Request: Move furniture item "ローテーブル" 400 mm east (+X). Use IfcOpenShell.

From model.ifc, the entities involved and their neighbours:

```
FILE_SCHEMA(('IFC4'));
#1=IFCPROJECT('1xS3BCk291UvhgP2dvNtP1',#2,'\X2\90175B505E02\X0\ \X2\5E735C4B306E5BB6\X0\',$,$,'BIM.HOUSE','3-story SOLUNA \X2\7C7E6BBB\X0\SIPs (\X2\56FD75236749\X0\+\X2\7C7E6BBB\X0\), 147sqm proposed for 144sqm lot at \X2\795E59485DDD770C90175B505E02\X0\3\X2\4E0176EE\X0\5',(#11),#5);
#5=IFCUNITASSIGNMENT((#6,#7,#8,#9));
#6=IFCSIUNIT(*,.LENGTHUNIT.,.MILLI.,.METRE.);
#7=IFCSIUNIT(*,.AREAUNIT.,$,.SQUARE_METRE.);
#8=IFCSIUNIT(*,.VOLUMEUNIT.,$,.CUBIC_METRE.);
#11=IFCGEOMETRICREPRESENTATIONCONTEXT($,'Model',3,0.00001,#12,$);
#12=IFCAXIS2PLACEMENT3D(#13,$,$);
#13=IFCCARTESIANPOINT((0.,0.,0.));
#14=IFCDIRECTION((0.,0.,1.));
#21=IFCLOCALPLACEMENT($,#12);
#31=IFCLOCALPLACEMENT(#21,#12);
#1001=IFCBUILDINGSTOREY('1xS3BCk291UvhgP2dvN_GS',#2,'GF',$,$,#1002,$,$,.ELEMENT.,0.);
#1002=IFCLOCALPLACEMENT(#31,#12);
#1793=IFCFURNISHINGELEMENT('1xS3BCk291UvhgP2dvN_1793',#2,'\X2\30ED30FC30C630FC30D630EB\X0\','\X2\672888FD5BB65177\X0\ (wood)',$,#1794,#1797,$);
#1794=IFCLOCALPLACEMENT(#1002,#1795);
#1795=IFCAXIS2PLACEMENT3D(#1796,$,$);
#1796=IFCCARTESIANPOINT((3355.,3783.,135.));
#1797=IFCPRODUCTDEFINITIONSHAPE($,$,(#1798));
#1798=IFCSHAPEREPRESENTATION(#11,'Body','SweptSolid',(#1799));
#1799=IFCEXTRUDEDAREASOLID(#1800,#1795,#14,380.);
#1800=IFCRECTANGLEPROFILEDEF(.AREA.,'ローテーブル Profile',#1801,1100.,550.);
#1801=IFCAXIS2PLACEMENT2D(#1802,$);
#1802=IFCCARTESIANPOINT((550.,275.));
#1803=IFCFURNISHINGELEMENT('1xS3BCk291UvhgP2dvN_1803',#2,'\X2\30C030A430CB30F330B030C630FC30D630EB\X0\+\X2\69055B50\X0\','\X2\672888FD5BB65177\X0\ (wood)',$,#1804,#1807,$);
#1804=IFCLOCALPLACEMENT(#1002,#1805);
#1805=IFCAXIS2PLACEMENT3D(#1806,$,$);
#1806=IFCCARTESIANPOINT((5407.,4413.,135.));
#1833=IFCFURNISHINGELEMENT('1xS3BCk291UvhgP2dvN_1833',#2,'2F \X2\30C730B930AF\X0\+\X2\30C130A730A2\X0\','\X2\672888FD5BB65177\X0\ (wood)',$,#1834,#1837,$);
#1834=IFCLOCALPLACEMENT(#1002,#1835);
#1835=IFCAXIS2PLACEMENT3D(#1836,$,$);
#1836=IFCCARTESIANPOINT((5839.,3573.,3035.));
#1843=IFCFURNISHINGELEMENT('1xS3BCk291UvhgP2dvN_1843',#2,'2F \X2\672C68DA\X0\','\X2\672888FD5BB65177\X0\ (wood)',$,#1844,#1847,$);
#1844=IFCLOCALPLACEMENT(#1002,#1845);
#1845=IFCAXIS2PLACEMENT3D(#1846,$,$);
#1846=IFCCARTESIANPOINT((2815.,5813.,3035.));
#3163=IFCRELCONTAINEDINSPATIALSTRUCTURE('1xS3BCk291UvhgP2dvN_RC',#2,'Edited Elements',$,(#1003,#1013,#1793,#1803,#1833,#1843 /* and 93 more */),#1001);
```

```python
import ifcopenshell
import ifcopenshell.api.geometry
import ifcopenshell.util.placement
import ifcopenshell.util.unit

model = ifcopenshell.open("model.ifc")
unit_scale = ifcopenshell.util.unit.calculate_unit_scale(model)

item = model.by_guid("1xS3BCk291UvhgP2dvN_1793")
matrix = ifcopenshell.util.placement.get_local_placement(item.ObjectPlacement)
matrix[0, 3] += 0.4 / unit_scale
ifcopenshell.api.geometry.edit_object_placement(model, product=item, matrix=matrix, is_si=False)

print(ifcopenshell.util.placement.get_local_placement(item.ObjectPlacement).round(3) + 0.0)

model.write("model-out.ifc")
```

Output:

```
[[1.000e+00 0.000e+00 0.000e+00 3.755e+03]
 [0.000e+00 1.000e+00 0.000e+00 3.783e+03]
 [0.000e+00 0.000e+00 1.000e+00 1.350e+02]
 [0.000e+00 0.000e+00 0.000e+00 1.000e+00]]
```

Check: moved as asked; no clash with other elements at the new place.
